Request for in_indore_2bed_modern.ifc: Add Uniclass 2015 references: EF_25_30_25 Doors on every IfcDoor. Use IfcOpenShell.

First a look at what the model holds.

```python
import ifcopenshell

model = ifcopenshell.open("in_indore_2bed_modern.ifc")
print(model.schema)
print("classifications:", [c.Name for c in model.by_type("IfcClassification")])
for ifc_class in ("IfcDoor", "IfcRoof", "IfcStair", "IfcWall", "IfcWindow"):
    print(ifc_class, len(model.by_type(ifc_class)))
```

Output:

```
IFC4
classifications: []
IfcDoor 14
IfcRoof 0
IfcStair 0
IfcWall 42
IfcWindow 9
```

```python
import ifcopenshell
import ifcopenshell.api.classification

model = ifcopenshell.open("in_indore_2bed_modern.ifc")

system = ifcopenshell.api.classification.add_classification(model, classification="Uniclass 2015")

codes = {
    "IfcDoor": ("EF_25_30_25", "Doors"),
}
for ifc_class, (code, name) in codes.items():
    products = model.by_type(ifc_class)
    ifcopenshell.api.classification.add_reference(
        model, products=products, classification=system, identification=code, name=name
    )
    print(code, len(products))

model.write("in_indore_2bed_modern-out.ifc")
```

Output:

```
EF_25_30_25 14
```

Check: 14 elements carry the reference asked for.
